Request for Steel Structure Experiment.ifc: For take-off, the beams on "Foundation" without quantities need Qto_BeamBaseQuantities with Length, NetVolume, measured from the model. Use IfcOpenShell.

First a look at what the model holds.

```python
import ifcopenshell
import ifcopenshell.util.element
import ifcopenshell.util.unit

model = ifcopenshell.open("Steel Structure Experiment.ifc")
print(model.schema)
for unit_type in ("LENGTHUNIT", "AREAUNIT", "VOLUMEUNIT"):
    print(unit_type, ifcopenshell.util.unit.calculate_unit_scale(model, unit_type))
storey = next(s for s in model.by_type("IfcBuildingStorey") if s.Name == "Foundation")
beams = [e for e in ifcopenshell.util.element.get_decomposition(storey) if e.is_a("IfcBeam")]
for e in sorted(beams, key=lambda e: e.id()):
    print(e.id(), e.is_a(), e.Name, list(ifcopenshell.util.element.get_psets(e, qtos_only=True)), sep=" | ")
```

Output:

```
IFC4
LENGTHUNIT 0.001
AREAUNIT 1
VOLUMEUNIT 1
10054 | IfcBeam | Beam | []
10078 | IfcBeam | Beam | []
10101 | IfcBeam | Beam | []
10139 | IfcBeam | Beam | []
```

```python
import ifcopenshell
import ifcopenshell.api.pset
import ifcopenshell.geom
import ifcopenshell.util.element
import ifcopenshell.util.shape
import ifcopenshell.util.unit

model = ifcopenshell.open("Steel Structure Experiment.ifc")
unit_scale = ifcopenshell.util.unit.calculate_unit_scale(model)
volume_scale = ifcopenshell.util.unit.calculate_unit_scale(model, "VOLUMEUNIT")
settings = ifcopenshell.geom.settings()

storey = next(s for s in model.by_type("IfcBuildingStorey") if s.Name == "Foundation")
beams = [e for e in ifcopenshell.util.element.get_decomposition(storey) if e.is_a("IfcBeam")]

for e in sorted(beams, key=lambda e: e.id()):
    if ifcopenshell.util.element.get_psets(e, qtos_only=True, should_inherit=False):
        continue
    # Geometry comes back in metres, in the element's own axes.
    shape = ifcopenshell.geom.create_shape(settings, e)
    values = {
        "Length": ifcopenshell.util.shape.get_max_xyz(shape.geometry) / unit_scale,
        "NetVolume": ifcopenshell.util.shape.get_volume(shape.geometry) / volume_scale,
    }
    qto = ifcopenshell.api.pset.add_qto(model, product=e, name="Qto_BeamBaseQuantities")
    ifcopenshell.api.pset.edit_qto(model, qto=qto, properties=values)
    print(e.id(), {k: round(v, 3) for k, v in values.items()})

model.write("Steel Structure Experiment_edited.ifc")
```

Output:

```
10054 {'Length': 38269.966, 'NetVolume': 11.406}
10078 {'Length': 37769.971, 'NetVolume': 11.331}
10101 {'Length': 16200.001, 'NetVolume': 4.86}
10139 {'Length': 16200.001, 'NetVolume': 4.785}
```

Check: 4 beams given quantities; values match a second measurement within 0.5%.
